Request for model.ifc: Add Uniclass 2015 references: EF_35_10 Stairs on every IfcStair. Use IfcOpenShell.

First a look at what the model holds.

```python
import ifcopenshell

model = ifcopenshell.open("model.ifc")
print(model.schema)
print("classifications:", [c.Name for c in model.by_type("IfcClassification")])
for ifc_class in ("IfcDoor", "IfcRoof", "IfcStair", "IfcWall", "IfcWindow"):
    print(ifc_class, len(model.by_type(ifc_class)))
```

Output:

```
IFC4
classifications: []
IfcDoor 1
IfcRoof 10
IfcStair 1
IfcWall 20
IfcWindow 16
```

```python
import ifcopenshell
import ifcopenshell.api.classification

model = ifcopenshell.open("model.ifc")

system = ifcopenshell.api.classification.add_classification(model, classification="Uniclass 2015")

codes = {
    "IfcStair": ("EF_35_10", "Stairs"),
}
for ifc_class, (code, name) in codes.items():
    products = model.by_type(ifc_class)
    ifcopenshell.api.classification.add_reference(
        model, products=products, classification=system, identification=code, name=name
    )
    print(code, len(products))

model.write("model_v2.ifc")
```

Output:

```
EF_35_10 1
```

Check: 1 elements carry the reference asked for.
